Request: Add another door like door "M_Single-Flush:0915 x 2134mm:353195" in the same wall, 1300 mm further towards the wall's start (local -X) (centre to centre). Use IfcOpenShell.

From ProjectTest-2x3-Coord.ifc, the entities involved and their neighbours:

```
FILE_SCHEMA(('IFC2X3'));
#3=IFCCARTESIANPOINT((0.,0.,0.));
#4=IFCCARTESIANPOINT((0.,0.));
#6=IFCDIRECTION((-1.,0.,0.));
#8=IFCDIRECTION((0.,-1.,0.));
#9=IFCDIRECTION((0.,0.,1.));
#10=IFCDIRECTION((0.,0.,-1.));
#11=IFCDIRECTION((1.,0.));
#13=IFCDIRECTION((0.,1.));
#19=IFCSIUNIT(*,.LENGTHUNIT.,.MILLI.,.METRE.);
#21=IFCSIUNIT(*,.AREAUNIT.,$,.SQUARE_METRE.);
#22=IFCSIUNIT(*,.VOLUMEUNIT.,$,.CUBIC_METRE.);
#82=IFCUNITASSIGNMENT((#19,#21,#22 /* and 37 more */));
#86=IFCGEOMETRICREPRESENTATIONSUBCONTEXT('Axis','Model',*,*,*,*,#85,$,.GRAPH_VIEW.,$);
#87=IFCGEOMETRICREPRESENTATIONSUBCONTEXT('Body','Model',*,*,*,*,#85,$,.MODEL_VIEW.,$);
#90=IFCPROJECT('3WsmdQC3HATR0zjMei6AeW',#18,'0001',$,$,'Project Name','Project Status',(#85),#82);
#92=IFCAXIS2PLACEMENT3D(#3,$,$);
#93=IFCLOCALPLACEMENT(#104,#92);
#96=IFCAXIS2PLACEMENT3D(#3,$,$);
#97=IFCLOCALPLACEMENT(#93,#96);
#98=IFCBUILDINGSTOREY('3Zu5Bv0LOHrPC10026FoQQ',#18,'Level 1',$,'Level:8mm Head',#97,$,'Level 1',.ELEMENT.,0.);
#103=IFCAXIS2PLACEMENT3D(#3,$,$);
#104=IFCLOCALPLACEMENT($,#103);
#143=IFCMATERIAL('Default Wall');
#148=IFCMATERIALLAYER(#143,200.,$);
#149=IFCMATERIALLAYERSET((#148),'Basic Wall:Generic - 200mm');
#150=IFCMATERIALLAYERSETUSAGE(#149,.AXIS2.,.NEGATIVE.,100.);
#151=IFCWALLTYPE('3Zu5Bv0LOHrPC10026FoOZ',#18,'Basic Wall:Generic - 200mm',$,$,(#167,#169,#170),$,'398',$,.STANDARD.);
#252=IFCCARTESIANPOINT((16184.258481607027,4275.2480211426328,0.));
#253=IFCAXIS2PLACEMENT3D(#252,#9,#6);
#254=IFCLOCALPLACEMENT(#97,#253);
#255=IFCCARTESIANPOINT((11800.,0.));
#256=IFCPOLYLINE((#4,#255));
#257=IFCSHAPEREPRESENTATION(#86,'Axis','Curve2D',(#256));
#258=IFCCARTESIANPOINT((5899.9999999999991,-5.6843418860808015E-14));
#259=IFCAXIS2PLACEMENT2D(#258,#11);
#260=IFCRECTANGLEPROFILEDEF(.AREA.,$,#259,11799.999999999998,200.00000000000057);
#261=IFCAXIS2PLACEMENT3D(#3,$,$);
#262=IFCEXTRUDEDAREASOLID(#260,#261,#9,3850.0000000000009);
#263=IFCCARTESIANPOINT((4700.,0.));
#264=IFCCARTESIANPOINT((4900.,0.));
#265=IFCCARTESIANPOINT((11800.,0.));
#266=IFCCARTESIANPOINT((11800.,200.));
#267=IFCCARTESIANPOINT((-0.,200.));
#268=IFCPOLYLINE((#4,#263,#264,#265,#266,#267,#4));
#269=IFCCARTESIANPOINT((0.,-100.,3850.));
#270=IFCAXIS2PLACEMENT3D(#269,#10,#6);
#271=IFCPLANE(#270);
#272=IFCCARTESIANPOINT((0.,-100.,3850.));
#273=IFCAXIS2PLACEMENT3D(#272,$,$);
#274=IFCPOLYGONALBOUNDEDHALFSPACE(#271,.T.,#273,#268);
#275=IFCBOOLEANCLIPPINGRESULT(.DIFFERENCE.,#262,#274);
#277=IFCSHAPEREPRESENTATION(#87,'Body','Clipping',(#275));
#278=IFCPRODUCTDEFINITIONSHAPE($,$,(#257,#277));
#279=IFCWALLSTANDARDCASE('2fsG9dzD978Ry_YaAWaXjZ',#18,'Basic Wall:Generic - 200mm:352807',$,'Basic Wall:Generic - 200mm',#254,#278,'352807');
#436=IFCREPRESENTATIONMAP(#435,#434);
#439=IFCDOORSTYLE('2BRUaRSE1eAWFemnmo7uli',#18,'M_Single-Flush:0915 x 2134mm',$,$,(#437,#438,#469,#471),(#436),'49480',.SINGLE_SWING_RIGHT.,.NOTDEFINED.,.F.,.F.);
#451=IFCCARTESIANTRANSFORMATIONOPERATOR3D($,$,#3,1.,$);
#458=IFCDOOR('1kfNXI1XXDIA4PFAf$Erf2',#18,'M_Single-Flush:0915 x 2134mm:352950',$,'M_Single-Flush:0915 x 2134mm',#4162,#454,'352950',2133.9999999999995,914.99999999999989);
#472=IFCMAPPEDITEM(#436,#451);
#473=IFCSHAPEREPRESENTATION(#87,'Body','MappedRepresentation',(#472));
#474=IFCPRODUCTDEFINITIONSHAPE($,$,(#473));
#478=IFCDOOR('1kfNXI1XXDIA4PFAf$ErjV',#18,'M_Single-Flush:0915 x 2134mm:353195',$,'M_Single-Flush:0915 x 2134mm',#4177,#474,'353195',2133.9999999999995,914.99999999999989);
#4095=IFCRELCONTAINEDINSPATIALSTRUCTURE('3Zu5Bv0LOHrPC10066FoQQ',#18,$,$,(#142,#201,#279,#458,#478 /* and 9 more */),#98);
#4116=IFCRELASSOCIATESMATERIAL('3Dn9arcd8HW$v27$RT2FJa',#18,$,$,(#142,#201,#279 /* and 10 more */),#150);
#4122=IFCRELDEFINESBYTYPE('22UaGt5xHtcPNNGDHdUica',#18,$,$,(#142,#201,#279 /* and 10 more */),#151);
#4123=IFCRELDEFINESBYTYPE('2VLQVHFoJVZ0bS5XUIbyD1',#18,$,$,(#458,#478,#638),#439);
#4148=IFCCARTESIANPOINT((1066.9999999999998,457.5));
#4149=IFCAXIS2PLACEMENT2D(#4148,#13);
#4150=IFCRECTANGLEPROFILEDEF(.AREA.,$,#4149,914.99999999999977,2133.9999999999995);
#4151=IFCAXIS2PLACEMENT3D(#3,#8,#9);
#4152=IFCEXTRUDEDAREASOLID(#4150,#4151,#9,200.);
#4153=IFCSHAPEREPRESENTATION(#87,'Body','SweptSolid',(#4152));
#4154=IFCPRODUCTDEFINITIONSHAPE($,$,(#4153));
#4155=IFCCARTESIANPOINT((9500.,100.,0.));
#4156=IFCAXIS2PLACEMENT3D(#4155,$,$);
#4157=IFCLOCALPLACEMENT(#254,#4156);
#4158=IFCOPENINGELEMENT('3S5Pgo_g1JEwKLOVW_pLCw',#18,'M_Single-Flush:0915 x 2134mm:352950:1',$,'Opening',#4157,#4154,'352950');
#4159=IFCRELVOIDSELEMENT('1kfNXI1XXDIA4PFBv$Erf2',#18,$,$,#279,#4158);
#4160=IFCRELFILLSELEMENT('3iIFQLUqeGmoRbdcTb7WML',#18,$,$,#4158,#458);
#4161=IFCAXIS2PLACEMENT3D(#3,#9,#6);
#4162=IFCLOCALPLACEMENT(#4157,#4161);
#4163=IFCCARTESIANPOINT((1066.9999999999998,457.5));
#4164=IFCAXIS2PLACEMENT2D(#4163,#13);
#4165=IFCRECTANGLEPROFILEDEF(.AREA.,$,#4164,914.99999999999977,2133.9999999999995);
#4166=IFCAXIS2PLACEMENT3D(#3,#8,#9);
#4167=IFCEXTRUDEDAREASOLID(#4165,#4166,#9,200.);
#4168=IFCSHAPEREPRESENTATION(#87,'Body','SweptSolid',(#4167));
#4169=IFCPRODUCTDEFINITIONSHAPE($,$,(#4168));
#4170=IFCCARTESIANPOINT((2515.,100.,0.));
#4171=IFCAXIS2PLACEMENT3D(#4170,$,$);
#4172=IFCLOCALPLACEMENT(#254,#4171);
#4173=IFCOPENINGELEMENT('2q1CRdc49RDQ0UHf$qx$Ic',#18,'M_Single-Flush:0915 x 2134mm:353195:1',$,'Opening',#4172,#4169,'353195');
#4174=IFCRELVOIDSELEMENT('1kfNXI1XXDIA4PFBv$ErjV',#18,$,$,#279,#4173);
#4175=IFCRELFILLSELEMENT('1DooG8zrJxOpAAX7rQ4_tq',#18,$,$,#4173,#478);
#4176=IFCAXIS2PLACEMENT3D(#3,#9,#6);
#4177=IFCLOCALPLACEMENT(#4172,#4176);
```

```python
import ifcopenshell
import ifcopenshell.api.feature
import ifcopenshell.api.geometry
import ifcopenshell.api.root
import ifcopenshell.geom
import ifcopenshell.util.element
import ifcopenshell.util.placement
import ifcopenshell.util.shape
import ifcopenshell.util.unit

model = ifcopenshell.open("ProjectTest-2x3-Coord.ifc")
unit_scale = ifcopenshell.util.unit.calculate_unit_scale(model)
settings = ifcopenshell.geom.settings()


def volume(element):
    """Net volume in cubic metres, openings subtracted."""
    shape = ifcopenshell.geom.create_shape(settings, element)
    return ifcopenshell.util.shape.get_volume(shape.geometry)


def reuse_history(source, copy):
    """copy_class also copies each property set's owner history, people and application; keep the originals."""
    for rel in copy.IsDefinedBy:
        if rel.is_a("IfcRelDefinesByProperties") and (history := rel.RelatingPropertyDefinition.OwnerHistory):
            rel.RelatingPropertyDefinition.OwnerHistory = source.OwnerHistory
            ifcopenshell.util.element.remove_deep2(model, history)


door = model.by_guid("1kfNXI1XXDIA4PFAf$ErjV")
opening = door.FillsVoids[0].RelatingOpeningElement
wall = opening.VoidsElements[0].RelatingBuildingElement
before = volume(wall)
shift = ifcopenshell.util.placement.get_local_placement(wall.ObjectPlacement)[:3, 0] * -1.3 / unit_scale

# copy_class copies the void relationship, type, container and properties, but no geometry.
new_opening = ifcopenshell.api.root.copy_class(model, product=opening)
new_opening.Representation = ifcopenshell.util.element.copy_deep(
    model, opening.Representation, exclude=["IfcGeometricRepresentationContext", "IfcRepresentationMap"]
)
new_opening.Name = "M_Single-Flush:0915 x 2134mm"
new_opening.Tag = None
new_door = ifcopenshell.api.root.copy_class(model, product=door)
new_door.Representation = ifcopenshell.util.element.copy_deep(
    model, door.Representation, exclude=["IfcGeometricRepresentationContext", "IfcRepresentationMap"]
)
new_door.Name = "M_Single-Flush:0915 x 2134mm"
new_door.Tag = None
reuse_history(door, new_door)
fills = ifcopenshell.api.feature.add_filling(model, opening=new_opening, element=new_door)
fills.OwnerHistory = new_door.OwnerHistory  # required in IFC2X3

for old, new in ((opening, new_opening), (door, new_door)):
    matrix = ifcopenshell.util.placement.get_local_placement(old.ObjectPlacement)
    matrix[:3, 3] += shift
    ifcopenshell.api.geometry.edit_object_placement(model, product=new, matrix=matrix, is_si=False)

after = volume(wall)

print(f"wall volume {before:.3f} -> {after:.3f} m3")

model.write("ProjectTest-2x3-Coord_rev.ifc")
```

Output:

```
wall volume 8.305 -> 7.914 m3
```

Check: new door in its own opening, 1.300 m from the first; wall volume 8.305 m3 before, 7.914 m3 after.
